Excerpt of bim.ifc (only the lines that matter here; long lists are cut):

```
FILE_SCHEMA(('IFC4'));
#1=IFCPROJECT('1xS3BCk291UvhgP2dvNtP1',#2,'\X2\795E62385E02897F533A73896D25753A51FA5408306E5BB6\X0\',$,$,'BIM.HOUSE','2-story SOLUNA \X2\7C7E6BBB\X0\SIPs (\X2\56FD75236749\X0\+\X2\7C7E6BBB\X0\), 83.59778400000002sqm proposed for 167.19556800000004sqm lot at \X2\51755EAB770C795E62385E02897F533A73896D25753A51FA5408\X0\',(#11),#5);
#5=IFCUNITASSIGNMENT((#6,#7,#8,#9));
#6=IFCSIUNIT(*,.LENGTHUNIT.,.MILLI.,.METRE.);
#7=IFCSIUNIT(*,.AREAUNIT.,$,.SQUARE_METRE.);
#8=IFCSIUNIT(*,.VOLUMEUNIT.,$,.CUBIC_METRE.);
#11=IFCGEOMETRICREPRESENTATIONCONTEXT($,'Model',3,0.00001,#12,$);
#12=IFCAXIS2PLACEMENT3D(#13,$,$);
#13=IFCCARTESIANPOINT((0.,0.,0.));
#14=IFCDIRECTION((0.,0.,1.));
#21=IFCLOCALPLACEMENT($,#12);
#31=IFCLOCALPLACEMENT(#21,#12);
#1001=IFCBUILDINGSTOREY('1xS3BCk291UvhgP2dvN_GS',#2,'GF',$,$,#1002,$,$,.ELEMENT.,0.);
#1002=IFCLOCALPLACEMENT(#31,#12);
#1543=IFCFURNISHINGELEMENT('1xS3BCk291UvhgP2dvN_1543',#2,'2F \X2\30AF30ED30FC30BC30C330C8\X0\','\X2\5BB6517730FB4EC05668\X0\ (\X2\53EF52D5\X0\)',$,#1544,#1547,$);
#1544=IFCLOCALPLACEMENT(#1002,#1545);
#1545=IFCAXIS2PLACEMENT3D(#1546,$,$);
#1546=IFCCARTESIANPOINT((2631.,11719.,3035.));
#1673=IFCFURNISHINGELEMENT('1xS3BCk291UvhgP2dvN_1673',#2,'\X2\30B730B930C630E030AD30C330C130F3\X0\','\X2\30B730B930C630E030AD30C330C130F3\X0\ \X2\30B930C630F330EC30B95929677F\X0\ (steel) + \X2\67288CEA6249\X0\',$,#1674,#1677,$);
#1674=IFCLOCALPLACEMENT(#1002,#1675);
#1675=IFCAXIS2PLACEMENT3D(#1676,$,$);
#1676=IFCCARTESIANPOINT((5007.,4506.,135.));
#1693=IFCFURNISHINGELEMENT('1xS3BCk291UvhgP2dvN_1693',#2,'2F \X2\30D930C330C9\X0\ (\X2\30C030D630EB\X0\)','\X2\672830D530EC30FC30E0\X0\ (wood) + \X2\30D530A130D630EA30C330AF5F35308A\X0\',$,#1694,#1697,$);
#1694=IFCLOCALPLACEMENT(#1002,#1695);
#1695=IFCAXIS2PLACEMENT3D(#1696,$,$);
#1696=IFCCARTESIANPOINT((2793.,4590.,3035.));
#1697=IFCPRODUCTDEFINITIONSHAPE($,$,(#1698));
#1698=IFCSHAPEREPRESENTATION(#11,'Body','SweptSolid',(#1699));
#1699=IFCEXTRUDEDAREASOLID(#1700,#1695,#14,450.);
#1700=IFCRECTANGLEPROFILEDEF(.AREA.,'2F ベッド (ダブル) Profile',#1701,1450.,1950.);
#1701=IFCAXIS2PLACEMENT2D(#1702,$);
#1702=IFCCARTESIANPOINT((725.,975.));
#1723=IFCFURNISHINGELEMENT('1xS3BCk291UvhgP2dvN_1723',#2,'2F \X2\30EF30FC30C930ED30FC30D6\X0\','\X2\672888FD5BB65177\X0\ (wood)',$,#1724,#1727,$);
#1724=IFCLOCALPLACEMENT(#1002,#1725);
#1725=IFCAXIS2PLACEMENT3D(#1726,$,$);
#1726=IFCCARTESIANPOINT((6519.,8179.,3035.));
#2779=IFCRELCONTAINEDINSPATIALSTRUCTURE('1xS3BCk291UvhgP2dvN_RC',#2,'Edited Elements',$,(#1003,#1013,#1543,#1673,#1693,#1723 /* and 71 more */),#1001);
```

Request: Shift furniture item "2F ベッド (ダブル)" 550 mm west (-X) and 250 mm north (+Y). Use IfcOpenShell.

```python
import ifcopenshell
import ifcopenshell.api.geometry
import ifcopenshell.util.placement
import ifcopenshell.util.unit

model = ifcopenshell.open("bim.ifc")
unit_scale = ifcopenshell.util.unit.calculate_unit_scale(model)

item = model.by_guid("1xS3BCk291UvhgP2dvN_1693")
matrix = ifcopenshell.util.placement.get_local_placement(item.ObjectPlacement)
matrix[0, 3] -= 0.55 / unit_scale
matrix[1, 3] += 0.25 / unit_scale
ifcopenshell.api.geometry.edit_object_placement(model, product=item, matrix=matrix, is_si=False)

print(ifcopenshell.util.placement.get_local_placement(item.ObjectPlacement).round(3) + 0.0)

model.write("bim_rev.ifc")
```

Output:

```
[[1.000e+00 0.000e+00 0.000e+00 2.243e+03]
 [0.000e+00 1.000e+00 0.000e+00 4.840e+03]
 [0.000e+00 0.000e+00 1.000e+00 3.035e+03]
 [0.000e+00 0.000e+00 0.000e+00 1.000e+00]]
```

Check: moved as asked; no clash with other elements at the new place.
